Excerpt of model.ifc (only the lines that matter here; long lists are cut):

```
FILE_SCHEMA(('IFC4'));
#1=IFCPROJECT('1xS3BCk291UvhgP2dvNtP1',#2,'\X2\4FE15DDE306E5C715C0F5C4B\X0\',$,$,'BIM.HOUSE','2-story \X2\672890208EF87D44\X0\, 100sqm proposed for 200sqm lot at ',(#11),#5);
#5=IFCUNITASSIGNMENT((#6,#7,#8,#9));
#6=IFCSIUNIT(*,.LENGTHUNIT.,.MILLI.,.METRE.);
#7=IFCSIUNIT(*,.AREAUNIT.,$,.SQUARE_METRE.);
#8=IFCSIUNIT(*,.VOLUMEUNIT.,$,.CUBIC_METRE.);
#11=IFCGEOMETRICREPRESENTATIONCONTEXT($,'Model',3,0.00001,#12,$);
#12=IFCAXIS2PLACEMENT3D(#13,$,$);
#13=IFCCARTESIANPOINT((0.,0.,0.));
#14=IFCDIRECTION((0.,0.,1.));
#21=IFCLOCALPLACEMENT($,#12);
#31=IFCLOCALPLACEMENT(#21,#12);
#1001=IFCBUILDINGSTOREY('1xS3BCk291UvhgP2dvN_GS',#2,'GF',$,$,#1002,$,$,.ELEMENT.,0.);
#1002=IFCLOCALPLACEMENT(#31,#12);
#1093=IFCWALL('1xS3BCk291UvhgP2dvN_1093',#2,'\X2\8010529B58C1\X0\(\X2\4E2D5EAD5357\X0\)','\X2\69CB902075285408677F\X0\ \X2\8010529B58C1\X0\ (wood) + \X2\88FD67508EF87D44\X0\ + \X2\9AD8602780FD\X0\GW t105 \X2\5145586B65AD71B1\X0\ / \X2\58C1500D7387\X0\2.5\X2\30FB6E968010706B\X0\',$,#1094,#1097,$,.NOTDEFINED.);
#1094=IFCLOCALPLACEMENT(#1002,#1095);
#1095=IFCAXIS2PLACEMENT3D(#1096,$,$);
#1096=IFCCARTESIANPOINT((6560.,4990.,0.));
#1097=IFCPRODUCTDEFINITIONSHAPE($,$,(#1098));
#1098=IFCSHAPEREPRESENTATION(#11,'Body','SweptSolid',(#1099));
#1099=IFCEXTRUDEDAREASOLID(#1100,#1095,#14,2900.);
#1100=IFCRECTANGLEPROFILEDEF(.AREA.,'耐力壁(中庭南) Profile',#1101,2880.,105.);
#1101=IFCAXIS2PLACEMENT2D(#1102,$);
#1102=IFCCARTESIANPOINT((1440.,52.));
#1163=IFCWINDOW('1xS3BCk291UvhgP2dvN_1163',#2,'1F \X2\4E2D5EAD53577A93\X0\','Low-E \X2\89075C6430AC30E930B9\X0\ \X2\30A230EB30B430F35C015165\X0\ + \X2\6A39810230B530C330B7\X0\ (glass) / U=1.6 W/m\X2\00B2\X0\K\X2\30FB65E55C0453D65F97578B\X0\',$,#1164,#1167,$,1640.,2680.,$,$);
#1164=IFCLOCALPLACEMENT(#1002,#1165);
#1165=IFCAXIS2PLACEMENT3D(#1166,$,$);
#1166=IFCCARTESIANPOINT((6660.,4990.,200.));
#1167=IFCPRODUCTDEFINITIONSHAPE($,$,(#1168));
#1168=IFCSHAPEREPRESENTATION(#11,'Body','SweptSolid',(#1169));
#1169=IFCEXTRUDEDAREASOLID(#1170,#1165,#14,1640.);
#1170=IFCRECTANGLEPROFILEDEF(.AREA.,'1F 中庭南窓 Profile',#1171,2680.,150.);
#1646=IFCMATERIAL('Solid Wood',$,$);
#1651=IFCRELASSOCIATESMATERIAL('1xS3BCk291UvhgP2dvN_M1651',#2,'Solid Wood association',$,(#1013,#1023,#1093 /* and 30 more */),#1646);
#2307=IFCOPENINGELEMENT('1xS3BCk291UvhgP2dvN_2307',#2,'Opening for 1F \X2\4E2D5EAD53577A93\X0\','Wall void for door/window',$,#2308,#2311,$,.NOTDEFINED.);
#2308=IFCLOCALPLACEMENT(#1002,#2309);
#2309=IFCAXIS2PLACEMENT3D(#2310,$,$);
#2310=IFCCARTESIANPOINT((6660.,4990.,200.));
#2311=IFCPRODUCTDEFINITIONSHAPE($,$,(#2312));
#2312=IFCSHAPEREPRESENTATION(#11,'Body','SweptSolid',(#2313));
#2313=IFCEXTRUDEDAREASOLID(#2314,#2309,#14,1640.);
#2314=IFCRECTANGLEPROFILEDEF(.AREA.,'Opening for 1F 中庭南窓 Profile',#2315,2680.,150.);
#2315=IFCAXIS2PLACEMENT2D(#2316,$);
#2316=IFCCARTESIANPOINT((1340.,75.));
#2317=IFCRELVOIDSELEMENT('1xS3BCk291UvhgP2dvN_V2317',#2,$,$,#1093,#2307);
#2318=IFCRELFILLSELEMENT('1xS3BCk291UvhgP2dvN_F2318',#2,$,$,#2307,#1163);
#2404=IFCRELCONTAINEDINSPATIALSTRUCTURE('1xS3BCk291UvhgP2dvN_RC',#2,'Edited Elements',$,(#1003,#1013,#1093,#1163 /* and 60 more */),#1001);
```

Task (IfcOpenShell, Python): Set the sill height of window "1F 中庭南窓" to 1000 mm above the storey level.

```python
import numpy as np
import ifcopenshell
import ifcopenshell.api.geometry
import ifcopenshell.geom
import ifcopenshell.util.element
import ifcopenshell.util.placement
import ifcopenshell.util.shape
import ifcopenshell.util.unit

model = ifcopenshell.open("model.ifc")
unit_scale = ifcopenshell.util.unit.calculate_unit_scale(model)

window = model.by_id(1163)
opening = window.FillsVoids[0].RelatingOpeningElement
storey = ifcopenshell.util.element.get_container(window, ifc_class="IfcBuildingStorey")
level = ifcopenshell.util.placement.get_local_placement(storey.ObjectPlacement)[2, 3]

# The opening's origin need not be at the sill, so measure its lowest point.
shape = ifcopenshell.geom.create_shape(ifcopenshell.geom.settings(), opening)
bottom = ifcopenshell.util.shape.get_shape_bottom_elevation(shape, shape.geometry) / unit_scale
dz = level + 1 / unit_scale - bottom

shift = np.array([0.0, 0.0, dz])
# The window is not placed relative to its opening, so move both.
for product in (opening, window):
    matrix = ifcopenshell.util.placement.get_local_placement(product.ObjectPlacement)
    matrix[:3, 3] += shift
    ifcopenshell.api.geometry.edit_object_placement(model, product=product, matrix=matrix, is_si=False)

print(f"moved by {dz * unit_scale:+.3f} m")

model.write("model_updated.ifc")
```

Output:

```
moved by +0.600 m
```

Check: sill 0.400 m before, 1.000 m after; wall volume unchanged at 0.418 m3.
